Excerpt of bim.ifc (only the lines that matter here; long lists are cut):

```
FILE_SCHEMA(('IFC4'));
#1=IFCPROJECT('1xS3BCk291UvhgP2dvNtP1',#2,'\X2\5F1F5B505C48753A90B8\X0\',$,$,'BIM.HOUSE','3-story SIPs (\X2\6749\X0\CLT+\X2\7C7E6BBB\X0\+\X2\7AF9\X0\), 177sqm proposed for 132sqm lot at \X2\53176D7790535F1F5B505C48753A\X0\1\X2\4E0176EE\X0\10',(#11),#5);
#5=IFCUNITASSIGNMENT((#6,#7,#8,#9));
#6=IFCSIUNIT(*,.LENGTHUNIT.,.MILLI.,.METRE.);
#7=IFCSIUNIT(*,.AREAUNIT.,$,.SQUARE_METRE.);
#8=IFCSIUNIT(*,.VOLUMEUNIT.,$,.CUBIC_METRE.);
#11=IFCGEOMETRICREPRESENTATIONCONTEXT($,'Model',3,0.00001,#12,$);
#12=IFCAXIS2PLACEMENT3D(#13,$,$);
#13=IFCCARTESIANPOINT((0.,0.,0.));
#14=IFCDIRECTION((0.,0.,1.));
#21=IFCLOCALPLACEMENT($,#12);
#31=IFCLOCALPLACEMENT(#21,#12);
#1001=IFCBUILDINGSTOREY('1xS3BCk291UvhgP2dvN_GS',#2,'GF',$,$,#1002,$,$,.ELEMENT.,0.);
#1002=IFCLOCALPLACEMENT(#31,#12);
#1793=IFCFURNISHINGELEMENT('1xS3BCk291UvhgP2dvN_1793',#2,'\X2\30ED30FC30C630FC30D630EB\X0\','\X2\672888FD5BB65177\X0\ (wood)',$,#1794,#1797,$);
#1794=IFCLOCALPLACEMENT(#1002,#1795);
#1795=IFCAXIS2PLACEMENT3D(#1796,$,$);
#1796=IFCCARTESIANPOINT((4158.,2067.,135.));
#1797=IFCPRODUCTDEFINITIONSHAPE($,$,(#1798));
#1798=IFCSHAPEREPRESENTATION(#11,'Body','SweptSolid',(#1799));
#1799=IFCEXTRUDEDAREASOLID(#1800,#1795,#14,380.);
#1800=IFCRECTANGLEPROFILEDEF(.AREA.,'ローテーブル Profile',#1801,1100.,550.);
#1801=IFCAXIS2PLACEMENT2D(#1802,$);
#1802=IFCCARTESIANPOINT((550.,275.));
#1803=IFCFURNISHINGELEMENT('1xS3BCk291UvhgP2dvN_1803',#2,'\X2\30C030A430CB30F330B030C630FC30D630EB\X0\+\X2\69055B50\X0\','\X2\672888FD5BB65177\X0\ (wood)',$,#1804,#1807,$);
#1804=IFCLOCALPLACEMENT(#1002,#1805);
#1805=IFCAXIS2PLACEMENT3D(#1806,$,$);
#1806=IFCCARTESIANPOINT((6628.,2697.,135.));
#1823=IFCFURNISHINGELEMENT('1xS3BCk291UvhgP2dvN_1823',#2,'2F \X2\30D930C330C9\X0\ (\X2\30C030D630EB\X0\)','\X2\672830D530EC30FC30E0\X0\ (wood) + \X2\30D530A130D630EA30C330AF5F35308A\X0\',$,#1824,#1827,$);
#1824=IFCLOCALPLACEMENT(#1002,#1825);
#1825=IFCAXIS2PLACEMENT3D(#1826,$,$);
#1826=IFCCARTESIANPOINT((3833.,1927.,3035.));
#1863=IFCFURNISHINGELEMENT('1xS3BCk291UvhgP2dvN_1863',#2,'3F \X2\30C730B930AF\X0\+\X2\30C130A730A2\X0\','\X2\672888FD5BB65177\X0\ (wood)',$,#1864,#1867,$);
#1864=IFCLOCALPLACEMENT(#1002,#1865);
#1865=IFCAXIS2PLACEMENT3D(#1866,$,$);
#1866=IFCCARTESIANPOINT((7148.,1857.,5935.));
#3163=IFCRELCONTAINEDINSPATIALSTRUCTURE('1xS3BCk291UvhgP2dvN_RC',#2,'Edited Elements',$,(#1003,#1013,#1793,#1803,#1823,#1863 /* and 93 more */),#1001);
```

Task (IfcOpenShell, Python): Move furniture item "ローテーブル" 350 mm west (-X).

```python
import ifcopenshell
import ifcopenshell.api.geometry
import ifcopenshell.util.placement

model = ifcopenshell.open("bim.ifc")

item = model.by_id(1793)
matrix = ifcopenshell.util.placement.get_local_placement(item.ObjectPlacement)
matrix[0, 3] -= 350.0
ifcopenshell.api.geometry.edit_object_placement(model, product=item, matrix=matrix, is_si=False)

print(ifcopenshell.util.placement.get_local_placement(item.ObjectPlacement).round(3) + 0.0)

model.write("bim_updated.ifc")
```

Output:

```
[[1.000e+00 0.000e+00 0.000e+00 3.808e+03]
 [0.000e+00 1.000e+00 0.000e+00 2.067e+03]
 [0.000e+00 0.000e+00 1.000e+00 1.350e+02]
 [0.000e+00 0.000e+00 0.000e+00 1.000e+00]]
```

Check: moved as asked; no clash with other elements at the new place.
